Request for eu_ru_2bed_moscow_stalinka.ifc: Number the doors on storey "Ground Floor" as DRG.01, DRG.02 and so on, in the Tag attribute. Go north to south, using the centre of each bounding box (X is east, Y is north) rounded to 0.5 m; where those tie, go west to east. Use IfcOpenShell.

First a look at what the model holds.

```python
import ifcopenshell
import ifcopenshell.util.element
import ifcopenshell.util.placement

model = ifcopenshell.open("eu_ru_2bed_moscow_stalinka.ifc")
print(model.schema)
storey = next(s for s in model.by_type("IfcBuildingStorey") if s.Name == "Ground Floor")
doors = [e for e in ifcopenshell.util.element.get_decomposition(storey) if e.is_a("IfcDoor")]
for e in sorted(doors, key=lambda e: e.id()):
    origin = ifcopenshell.util.placement.get_local_placement(e.ObjectPlacement)[:3, 3]
    print(e.id(), e.Tag, e.Name, origin.round(2) + 0.0, sep=" | ")
```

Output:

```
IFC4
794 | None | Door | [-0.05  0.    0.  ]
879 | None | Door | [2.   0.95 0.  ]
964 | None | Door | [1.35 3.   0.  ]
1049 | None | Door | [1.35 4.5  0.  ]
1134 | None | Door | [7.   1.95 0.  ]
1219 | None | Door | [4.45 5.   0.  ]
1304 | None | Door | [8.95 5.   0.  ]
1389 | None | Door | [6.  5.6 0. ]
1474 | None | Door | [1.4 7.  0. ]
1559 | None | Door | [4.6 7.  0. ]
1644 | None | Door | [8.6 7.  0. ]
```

```python
import ifcopenshell
import ifcopenshell.geom
import ifcopenshell.util.element
import ifcopenshell.util.shape

model = ifcopenshell.open("eu_ru_2bed_moscow_stalinka.ifc")
settings = ifcopenshell.geom.settings()
settings.set("use-world-coords", True)


def centre(element):
    shape = ifcopenshell.geom.create_shape(settings, element)
    return ifcopenshell.util.shape.get_bbox_centroid(shape.geometry)


storey = next(s for s in model.by_type("IfcBuildingStorey") if s.Name == "Ground Floor")
doors = [e for e in ifcopenshell.util.element.get_decomposition(storey) if e.is_a("IfcDoor")]

# Insertion points can sit at a corner or the storey origin, so sort by the geometry (in metres).
centres = {e: centre(e) for e in doors}
doors.sort(key=lambda e: (-round(centres[e][1] / 0.5), centres[e][0]))

for i, e in enumerate(doors, start=1):
    number = f"DRG.{i:02d}"
    e.Tag = number
    print(e.id(), number)

model.write("eu_ru_2bed_moscow_stalinka_rev.ifc")
```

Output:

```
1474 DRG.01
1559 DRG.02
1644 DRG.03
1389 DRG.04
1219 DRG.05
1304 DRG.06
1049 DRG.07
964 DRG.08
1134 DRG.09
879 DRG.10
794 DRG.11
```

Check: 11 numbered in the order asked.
